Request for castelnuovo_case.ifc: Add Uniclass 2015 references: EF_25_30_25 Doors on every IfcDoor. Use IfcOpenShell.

First a look at what the model holds.

```python
import ifcopenshell

model = ifcopenshell.open("castelnuovo_case.ifc")
print(model.schema)
print("classifications:", [c.Name for c in model.by_type("IfcClassification")])
for ifc_class in ("IfcDoor", "IfcRoof", "IfcStair", "IfcWall", "IfcWindow"):
    print(ifc_class, len(model.by_type(ifc_class)))
```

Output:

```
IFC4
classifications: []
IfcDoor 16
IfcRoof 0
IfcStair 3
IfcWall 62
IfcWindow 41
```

```python
import ifcopenshell
import ifcopenshell.api.classification

model = ifcopenshell.open("castelnuovo_case.ifc")

system = ifcopenshell.api.classification.add_classification(model, classification="Uniclass 2015")

codes = {
    "IfcDoor": ("EF_25_30_25", "Doors"),
}
for ifc_class, (code, name) in codes.items():
    products = model.by_type(ifc_class)
    ifcopenshell.api.classification.add_reference(
        model, products=products, classification=system, identification=code, name=name
    )
    print(code, len(products))

model.write("castelnuovo_case-out.ifc")
```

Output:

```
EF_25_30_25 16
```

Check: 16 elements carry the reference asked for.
